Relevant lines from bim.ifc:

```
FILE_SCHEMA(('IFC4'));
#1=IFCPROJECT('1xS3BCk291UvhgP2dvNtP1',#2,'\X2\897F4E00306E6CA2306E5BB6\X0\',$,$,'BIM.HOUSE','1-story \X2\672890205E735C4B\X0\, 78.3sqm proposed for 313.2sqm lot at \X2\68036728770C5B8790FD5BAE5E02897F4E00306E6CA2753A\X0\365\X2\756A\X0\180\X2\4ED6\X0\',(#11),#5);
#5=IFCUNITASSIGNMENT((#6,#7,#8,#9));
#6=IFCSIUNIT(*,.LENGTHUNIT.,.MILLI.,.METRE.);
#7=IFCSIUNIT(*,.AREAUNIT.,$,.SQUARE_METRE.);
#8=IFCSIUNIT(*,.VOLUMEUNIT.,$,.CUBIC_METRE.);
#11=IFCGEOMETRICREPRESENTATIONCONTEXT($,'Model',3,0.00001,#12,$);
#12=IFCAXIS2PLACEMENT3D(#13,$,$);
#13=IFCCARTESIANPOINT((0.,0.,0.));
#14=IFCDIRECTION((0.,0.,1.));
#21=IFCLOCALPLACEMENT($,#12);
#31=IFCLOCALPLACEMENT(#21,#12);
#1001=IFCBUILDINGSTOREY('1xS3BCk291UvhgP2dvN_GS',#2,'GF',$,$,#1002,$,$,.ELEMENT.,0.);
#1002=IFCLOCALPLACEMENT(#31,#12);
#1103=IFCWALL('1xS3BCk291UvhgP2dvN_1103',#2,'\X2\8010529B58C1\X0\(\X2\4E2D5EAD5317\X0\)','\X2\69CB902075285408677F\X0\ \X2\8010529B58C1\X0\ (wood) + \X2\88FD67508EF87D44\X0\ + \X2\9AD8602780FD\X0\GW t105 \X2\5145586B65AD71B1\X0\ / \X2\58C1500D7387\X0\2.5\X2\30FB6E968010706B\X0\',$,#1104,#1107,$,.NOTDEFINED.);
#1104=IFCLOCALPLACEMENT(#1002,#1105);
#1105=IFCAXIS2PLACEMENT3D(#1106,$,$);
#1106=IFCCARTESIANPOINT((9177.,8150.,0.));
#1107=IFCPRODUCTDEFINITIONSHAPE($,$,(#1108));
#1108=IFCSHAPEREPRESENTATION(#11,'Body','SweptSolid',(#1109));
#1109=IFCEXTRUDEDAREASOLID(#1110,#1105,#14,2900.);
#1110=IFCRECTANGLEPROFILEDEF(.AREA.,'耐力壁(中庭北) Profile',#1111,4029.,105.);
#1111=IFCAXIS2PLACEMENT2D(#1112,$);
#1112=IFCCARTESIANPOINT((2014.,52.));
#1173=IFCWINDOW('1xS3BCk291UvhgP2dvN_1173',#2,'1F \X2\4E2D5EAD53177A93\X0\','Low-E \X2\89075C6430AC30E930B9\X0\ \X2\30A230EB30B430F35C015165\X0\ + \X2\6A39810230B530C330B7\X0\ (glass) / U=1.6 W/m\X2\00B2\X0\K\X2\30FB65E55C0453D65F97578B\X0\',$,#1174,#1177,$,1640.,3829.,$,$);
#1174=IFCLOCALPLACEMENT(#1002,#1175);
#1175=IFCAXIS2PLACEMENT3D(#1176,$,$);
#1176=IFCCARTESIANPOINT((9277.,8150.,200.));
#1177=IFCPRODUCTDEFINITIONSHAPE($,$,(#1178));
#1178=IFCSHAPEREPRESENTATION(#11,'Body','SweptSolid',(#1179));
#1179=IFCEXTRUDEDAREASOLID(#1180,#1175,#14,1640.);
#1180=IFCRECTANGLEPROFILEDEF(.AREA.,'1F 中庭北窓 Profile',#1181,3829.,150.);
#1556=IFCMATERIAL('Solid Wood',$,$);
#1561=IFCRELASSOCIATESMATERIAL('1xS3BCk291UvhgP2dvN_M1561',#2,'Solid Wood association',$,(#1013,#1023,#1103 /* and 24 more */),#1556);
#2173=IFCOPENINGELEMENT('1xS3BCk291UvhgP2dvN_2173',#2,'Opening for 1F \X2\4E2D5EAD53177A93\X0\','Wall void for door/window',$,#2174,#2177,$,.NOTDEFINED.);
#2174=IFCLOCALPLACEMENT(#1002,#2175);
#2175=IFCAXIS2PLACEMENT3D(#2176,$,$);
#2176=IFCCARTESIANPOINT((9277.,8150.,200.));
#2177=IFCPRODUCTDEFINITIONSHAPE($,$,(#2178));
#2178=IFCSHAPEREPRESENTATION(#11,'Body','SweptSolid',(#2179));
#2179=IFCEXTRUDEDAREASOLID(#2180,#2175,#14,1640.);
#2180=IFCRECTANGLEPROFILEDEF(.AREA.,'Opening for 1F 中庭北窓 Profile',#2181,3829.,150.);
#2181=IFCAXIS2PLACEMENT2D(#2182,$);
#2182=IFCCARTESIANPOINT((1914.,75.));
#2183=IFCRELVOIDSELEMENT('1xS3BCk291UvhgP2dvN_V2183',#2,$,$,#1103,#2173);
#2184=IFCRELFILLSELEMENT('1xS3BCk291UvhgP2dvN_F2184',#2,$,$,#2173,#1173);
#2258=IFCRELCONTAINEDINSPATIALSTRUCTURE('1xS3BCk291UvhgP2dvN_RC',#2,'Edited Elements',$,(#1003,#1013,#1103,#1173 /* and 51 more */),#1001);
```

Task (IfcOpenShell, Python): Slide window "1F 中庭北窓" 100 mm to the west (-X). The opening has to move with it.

```python
import ifcopenshell
import ifcopenshell.api.geometry
import ifcopenshell.util.placement

model = ifcopenshell.open("bim.ifc")

window = model.by_guid("1xS3BCk291UvhgP2dvN_1173")
opening = window.FillsVoids[0].RelatingOpeningElement
wall = opening.VoidsElements[0].RelatingBuildingElement

wall_matrix = ifcopenshell.util.placement.get_local_placement(wall.ObjectPlacement)
shift = wall_matrix[:3, 0] * -100.0
before = ifcopenshell.util.placement.get_local_placement(window.ObjectPlacement)[:3, 3].copy()

# The window is not placed relative to its opening, so move both.
for product in (opening, window):
    matrix = ifcopenshell.util.placement.get_local_placement(product.ObjectPlacement)
    matrix[:3, 3] += shift
    ifcopenshell.api.geometry.edit_object_placement(model, product=product, matrix=matrix, is_si=False)

after = ifcopenshell.util.placement.get_local_placement(window.ObjectPlacement)[:3, 3]
print("window moved by", (after - before).round(3) + 0.0)

model.write("bim-out.ifc")
```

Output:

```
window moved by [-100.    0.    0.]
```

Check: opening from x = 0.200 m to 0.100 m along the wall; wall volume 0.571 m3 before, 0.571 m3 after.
